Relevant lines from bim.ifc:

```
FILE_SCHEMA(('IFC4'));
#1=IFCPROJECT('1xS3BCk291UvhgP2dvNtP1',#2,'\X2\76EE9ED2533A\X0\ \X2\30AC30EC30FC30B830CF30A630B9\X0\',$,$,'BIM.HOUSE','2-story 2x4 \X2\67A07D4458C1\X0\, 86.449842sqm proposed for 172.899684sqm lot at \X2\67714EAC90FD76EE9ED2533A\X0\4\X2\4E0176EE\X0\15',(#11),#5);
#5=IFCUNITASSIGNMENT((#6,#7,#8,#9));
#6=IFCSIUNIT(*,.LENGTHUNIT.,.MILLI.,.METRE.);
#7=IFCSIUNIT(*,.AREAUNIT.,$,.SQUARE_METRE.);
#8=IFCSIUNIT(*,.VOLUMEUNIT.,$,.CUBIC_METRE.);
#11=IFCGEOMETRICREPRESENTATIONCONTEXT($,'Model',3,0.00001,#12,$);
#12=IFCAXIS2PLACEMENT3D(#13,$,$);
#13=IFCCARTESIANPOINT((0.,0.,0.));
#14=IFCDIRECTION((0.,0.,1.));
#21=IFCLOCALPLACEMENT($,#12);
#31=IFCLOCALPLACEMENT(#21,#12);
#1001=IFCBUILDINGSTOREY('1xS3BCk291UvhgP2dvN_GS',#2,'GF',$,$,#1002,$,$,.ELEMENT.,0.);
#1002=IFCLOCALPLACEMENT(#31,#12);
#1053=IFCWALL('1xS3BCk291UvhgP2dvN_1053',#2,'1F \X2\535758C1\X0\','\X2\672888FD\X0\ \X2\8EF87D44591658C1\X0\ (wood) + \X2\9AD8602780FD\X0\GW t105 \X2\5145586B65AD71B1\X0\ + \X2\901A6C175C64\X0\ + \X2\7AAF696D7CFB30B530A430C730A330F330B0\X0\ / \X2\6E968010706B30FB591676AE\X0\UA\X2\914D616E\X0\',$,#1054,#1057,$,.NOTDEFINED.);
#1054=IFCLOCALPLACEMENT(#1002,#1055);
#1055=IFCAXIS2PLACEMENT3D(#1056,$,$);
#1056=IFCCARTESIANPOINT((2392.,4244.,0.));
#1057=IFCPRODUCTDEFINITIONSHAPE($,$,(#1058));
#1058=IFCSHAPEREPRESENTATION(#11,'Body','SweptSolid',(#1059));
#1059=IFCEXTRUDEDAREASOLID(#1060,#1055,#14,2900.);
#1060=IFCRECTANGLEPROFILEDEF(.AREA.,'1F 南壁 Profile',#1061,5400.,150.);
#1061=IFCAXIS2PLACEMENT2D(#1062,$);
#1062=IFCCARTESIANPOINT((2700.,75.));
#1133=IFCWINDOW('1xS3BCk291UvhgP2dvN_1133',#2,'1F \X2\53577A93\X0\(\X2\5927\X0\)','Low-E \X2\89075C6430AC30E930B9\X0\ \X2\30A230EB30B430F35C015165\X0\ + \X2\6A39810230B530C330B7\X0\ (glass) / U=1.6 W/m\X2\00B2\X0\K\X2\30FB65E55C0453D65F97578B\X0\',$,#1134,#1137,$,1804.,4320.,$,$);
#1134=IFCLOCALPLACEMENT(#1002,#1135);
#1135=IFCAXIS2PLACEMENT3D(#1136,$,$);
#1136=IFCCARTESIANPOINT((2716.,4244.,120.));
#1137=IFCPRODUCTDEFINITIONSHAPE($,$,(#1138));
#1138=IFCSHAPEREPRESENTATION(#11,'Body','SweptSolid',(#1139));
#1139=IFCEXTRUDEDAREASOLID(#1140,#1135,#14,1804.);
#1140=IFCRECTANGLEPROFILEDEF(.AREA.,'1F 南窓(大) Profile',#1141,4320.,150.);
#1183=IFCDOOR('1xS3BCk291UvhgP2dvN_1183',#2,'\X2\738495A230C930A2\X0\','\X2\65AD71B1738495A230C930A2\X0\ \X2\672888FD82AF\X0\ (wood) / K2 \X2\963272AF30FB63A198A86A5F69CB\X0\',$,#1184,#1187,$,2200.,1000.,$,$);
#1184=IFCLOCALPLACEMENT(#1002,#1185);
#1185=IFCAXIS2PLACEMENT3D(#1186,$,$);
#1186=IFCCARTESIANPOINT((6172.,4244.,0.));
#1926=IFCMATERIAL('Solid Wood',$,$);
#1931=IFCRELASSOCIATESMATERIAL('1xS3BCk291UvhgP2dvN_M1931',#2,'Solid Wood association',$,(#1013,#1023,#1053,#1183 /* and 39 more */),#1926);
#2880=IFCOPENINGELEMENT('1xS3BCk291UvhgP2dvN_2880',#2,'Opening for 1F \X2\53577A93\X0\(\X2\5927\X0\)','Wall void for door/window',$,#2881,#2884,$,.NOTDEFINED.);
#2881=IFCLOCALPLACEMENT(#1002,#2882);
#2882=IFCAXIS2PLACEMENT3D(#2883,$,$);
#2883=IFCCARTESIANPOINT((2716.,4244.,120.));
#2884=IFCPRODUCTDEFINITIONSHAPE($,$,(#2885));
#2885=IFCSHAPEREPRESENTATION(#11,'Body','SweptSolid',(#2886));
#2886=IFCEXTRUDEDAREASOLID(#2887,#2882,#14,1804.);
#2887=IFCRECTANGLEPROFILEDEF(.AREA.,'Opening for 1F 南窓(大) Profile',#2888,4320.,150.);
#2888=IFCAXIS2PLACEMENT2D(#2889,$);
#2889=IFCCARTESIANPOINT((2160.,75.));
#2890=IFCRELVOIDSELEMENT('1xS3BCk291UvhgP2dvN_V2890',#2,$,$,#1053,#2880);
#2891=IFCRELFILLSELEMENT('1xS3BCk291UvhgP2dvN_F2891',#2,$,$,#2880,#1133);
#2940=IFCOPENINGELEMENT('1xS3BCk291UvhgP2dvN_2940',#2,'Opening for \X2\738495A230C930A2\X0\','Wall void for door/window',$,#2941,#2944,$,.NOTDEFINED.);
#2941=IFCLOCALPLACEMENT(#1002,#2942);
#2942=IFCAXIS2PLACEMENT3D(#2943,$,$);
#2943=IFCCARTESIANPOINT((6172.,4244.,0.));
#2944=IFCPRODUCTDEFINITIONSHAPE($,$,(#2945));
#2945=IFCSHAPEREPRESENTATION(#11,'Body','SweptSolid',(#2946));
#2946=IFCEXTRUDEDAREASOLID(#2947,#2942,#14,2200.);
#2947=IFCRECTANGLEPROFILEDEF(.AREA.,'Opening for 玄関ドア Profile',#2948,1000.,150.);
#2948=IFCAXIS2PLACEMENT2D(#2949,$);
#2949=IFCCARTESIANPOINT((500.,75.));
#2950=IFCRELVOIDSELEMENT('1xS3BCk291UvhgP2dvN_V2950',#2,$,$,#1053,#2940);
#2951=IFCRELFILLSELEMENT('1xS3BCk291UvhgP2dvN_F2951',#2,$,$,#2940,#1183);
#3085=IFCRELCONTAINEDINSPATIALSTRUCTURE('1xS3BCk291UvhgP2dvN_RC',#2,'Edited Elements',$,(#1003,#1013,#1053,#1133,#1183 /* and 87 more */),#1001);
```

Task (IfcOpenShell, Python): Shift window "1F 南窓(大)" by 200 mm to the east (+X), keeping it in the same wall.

```python
import ifcopenshell
import ifcopenshell.api.geometry
import ifcopenshell.util.placement
import ifcopenshell.util.unit

model = ifcopenshell.open("bim.ifc")
unit_scale = ifcopenshell.util.unit.calculate_unit_scale(model)

window = model.by_id(1133)
opening = window.FillsVoids[0].RelatingOpeningElement
wall = opening.VoidsElements[0].RelatingBuildingElement

wall_matrix = ifcopenshell.util.placement.get_local_placement(wall.ObjectPlacement)
shift = wall_matrix[:3, 0] * 0.2 / unit_scale
before = ifcopenshell.util.placement.get_local_placement(window.ObjectPlacement)[:3, 3].copy()

# The window is not placed relative to its opening, so move both.
for product in (opening, window):
    matrix = ifcopenshell.util.placement.get_local_placement(product.ObjectPlacement)
    matrix[:3, 3] += shift
    ifcopenshell.api.geometry.edit_object_placement(model, product=product, matrix=matrix, is_si=False)

after = ifcopenshell.util.placement.get_local_placement(window.ObjectPlacement)[:3, 3]
print("window moved by", (after - before).round(3) + 0.0)

model.write("bim_edited.ifc")
```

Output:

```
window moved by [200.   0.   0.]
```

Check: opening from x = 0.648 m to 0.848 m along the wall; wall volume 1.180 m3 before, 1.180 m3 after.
